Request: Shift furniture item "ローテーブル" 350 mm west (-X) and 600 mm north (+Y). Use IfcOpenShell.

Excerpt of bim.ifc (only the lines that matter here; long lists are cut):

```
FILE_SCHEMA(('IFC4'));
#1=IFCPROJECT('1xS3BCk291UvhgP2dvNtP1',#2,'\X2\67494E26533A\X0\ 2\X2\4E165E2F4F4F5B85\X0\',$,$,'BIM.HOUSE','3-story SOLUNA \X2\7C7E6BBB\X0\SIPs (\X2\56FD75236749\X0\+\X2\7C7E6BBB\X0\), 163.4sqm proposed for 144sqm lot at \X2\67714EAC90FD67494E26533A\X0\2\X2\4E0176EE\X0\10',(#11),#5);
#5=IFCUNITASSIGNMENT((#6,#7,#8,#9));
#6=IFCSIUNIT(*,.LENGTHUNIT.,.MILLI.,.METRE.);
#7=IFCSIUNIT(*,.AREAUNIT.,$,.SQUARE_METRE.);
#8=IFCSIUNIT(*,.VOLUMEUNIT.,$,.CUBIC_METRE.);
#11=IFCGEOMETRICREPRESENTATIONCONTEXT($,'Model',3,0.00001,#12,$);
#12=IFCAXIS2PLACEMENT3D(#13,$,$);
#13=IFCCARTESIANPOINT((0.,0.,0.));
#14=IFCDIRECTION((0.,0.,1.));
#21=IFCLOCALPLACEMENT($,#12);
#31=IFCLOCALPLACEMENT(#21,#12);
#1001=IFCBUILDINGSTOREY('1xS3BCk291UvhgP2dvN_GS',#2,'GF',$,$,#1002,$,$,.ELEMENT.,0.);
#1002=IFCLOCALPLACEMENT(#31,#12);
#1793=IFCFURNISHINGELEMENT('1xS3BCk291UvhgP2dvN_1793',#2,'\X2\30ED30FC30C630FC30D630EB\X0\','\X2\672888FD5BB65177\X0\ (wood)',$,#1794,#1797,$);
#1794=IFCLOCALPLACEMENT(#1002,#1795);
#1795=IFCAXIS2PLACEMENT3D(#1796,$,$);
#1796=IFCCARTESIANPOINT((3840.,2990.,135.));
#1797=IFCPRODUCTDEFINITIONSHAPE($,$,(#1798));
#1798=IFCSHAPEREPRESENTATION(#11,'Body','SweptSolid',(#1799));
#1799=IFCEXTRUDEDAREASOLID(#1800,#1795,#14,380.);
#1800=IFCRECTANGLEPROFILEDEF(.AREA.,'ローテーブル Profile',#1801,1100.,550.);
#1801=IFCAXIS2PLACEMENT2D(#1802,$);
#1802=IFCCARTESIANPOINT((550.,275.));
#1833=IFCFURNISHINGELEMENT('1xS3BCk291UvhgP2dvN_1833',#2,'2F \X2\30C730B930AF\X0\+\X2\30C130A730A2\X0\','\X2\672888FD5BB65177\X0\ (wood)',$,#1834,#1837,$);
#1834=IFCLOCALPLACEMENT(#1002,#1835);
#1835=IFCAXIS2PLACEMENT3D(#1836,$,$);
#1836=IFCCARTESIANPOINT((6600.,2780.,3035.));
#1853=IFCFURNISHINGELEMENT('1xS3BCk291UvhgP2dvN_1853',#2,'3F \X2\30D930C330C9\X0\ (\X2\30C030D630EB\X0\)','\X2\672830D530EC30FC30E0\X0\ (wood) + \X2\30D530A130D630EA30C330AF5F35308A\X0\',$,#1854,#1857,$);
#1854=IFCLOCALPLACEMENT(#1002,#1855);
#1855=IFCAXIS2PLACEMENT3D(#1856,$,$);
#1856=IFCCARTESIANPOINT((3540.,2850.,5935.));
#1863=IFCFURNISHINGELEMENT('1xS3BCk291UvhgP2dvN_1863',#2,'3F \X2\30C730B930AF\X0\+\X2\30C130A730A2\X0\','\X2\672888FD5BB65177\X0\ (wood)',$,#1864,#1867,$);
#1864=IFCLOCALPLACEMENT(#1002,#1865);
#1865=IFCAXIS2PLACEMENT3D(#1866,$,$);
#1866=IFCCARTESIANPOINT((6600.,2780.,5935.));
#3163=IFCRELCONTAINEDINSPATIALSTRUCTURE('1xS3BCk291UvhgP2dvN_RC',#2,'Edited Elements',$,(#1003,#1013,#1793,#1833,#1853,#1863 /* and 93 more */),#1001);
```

```python
import ifcopenshell
import ifcopenshell.api.geometry
import ifcopenshell.util.placement

model = ifcopenshell.open("bim.ifc")

item = model.by_id(1793)
matrix = ifcopenshell.util.placement.get_local_placement(item.ObjectPlacement)
matrix[0, 3] -= 350.0
matrix[1, 3] += 600.0
ifcopenshell.api.geometry.edit_object_placement(model, product=item, matrix=matrix, is_si=False)

print(ifcopenshell.util.placement.get_local_placement(item.ObjectPlacement).round(3) + 0.0)

model.write("bim_v2.ifc")
```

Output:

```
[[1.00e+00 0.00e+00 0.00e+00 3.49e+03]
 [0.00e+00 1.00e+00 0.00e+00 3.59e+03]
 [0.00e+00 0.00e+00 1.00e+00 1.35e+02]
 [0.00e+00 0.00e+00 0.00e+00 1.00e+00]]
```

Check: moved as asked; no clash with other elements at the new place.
